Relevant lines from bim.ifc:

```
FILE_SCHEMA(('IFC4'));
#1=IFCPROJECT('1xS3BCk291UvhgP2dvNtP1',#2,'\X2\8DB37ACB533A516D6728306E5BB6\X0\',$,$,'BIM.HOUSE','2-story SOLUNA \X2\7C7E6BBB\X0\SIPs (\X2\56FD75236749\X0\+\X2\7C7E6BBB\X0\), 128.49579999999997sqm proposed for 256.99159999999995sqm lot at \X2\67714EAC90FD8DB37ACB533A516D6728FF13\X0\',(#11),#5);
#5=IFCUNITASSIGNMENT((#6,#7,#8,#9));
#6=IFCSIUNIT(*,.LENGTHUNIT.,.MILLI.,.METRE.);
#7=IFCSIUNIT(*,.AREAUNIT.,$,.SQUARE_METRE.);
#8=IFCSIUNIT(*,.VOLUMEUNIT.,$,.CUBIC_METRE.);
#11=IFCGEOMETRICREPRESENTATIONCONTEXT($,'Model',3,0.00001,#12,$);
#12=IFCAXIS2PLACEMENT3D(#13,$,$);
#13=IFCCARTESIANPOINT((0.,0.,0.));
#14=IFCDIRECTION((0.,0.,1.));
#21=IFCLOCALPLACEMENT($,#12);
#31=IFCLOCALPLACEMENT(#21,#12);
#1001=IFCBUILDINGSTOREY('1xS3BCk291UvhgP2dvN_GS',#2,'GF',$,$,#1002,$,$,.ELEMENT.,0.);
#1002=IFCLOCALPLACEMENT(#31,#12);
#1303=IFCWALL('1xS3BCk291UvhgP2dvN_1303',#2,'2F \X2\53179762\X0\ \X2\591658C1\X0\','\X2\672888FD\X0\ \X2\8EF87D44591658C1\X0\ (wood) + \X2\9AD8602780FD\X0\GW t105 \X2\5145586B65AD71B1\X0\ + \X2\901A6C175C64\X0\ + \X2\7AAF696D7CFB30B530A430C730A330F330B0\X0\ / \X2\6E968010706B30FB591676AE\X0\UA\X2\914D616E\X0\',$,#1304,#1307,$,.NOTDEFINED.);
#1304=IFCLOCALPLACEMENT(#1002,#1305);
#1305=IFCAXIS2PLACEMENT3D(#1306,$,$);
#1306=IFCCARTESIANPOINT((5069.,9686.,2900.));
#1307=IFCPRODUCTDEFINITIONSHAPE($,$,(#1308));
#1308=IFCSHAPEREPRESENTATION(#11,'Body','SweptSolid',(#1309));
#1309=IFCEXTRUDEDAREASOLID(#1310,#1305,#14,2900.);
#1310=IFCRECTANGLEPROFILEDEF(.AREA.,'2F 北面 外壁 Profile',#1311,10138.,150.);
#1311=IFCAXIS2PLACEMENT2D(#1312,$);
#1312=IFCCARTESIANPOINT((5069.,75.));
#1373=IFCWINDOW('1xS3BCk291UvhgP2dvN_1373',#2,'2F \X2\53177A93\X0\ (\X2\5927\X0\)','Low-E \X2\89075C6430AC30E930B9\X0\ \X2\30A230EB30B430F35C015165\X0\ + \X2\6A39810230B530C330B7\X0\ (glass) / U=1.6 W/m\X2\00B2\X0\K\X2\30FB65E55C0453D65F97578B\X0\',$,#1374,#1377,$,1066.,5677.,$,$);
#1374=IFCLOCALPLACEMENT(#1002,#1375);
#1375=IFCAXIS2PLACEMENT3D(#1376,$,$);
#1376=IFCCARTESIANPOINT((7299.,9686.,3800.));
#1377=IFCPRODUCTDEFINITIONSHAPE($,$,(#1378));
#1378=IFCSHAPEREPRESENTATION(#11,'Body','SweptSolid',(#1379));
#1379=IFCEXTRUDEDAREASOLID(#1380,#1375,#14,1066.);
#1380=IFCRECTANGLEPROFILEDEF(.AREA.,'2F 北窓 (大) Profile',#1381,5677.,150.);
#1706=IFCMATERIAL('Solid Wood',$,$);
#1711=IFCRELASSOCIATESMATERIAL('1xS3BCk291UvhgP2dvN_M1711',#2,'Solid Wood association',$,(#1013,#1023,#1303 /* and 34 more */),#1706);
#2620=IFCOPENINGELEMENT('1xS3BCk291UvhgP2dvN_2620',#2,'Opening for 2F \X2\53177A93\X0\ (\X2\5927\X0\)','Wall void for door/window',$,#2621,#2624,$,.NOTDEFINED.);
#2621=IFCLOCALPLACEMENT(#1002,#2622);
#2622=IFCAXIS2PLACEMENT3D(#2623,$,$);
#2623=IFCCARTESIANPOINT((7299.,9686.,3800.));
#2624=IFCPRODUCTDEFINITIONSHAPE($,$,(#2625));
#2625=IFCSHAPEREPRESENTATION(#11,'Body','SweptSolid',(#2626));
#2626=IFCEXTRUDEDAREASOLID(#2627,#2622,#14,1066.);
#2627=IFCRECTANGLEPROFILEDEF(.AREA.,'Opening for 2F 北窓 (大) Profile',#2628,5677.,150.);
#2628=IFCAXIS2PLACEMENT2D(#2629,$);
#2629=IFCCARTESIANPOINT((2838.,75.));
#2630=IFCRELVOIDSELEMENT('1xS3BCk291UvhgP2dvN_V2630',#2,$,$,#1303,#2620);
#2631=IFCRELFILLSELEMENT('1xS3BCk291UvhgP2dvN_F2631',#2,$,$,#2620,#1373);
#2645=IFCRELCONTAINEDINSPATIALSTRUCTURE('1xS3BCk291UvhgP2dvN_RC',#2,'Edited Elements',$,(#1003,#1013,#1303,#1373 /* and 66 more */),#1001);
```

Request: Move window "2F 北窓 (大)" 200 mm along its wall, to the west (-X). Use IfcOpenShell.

```python
import ifcopenshell
import ifcopenshell.api.geometry
import ifcopenshell.util.placement

model = ifcopenshell.open("bim.ifc")

window = model.by_guid("1xS3BCk291UvhgP2dvN_1373")
opening = window.FillsVoids[0].RelatingOpeningElement
wall = opening.VoidsElements[0].RelatingBuildingElement

wall_matrix = ifcopenshell.util.placement.get_local_placement(wall.ObjectPlacement)
shift = wall_matrix[:3, 0] * -200.0
before = ifcopenshell.util.placement.get_local_placement(window.ObjectPlacement)[:3, 3].copy()

# The window is not placed relative to its opening, so move both.
for product in (opening, window):
    matrix = ifcopenshell.util.placement.get_local_placement(product.ObjectPlacement)
    matrix[:3, 3] += shift
    ifcopenshell.api.geometry.edit_object_placement(model, product=product, matrix=matrix, is_si=False)

after = ifcopenshell.util.placement.get_local_placement(window.ObjectPlacement)[:3, 3]
print("window moved by", (after - before).round(3) + 0.0)

model.write("bim_edited.ifc")
```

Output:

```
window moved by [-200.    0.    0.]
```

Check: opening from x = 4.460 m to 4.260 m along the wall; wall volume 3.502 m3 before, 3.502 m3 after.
